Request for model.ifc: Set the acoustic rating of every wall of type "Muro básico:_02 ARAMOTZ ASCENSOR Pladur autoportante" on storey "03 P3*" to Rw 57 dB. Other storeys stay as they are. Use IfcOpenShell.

First a look at what the model holds.

```python
import ifcopenshell
import ifcopenshell.util.element

model = ifcopenshell.open("model.ifc")
print(model.schema)
storey = next(s for s in model.by_type("IfcBuildingStorey") if s.Name == "03 P3*")
walls = [e for e in ifcopenshell.util.element.get_decomposition(storey) if e.is_a("IfcWall")]
seen = {}
for e in walls:
    element_type = ifcopenshell.util.element.get_type(e)
    key = (element_type.Name if element_type != e and element_type else None, ifcopenshell.util.element.get_pset(e, "Pset_WallCommon", "AcousticRating"))
    seen[key] = seen.get(key, 0) + 1
for (name, value), count in sorted(seen.items(), key=str):
    print(count, "x", name, "|", value)
```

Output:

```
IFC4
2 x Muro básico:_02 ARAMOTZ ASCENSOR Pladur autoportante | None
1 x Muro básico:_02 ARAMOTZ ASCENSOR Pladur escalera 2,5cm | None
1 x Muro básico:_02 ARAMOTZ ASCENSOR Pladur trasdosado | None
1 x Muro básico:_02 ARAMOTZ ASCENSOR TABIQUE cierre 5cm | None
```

```python
import ifcopenshell
import ifcopenshell.api.pset
import ifcopenshell.util.element

model = ifcopenshell.open("model.ifc")

storey = next(s for s in model.by_type("IfcBuildingStorey") if s.Name == "03 P3*")
walls = [e for e in ifcopenshell.util.element.get_decomposition(storey) if e.is_a("IfcWall")]

count = 0
for e in walls:
    element_type = ifcopenshell.util.element.get_type(e)
    if element_type in (None, e) or element_type.Name != "Muro básico:_02 ARAMOTZ ASCENSOR Pladur autoportante":
        continue
    # add_pset returns the element's existing set when there is one.
    pset = ifcopenshell.api.pset.add_pset(model, product=e, name="Pset_WallCommon")
    ifcopenshell.api.pset.edit_pset(model, pset=pset, properties={"AcousticRating": "Rw 57 dB"})
    count += 1

print(count, "walls updated")

model.write("model-out.ifc")
```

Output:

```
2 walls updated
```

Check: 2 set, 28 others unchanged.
